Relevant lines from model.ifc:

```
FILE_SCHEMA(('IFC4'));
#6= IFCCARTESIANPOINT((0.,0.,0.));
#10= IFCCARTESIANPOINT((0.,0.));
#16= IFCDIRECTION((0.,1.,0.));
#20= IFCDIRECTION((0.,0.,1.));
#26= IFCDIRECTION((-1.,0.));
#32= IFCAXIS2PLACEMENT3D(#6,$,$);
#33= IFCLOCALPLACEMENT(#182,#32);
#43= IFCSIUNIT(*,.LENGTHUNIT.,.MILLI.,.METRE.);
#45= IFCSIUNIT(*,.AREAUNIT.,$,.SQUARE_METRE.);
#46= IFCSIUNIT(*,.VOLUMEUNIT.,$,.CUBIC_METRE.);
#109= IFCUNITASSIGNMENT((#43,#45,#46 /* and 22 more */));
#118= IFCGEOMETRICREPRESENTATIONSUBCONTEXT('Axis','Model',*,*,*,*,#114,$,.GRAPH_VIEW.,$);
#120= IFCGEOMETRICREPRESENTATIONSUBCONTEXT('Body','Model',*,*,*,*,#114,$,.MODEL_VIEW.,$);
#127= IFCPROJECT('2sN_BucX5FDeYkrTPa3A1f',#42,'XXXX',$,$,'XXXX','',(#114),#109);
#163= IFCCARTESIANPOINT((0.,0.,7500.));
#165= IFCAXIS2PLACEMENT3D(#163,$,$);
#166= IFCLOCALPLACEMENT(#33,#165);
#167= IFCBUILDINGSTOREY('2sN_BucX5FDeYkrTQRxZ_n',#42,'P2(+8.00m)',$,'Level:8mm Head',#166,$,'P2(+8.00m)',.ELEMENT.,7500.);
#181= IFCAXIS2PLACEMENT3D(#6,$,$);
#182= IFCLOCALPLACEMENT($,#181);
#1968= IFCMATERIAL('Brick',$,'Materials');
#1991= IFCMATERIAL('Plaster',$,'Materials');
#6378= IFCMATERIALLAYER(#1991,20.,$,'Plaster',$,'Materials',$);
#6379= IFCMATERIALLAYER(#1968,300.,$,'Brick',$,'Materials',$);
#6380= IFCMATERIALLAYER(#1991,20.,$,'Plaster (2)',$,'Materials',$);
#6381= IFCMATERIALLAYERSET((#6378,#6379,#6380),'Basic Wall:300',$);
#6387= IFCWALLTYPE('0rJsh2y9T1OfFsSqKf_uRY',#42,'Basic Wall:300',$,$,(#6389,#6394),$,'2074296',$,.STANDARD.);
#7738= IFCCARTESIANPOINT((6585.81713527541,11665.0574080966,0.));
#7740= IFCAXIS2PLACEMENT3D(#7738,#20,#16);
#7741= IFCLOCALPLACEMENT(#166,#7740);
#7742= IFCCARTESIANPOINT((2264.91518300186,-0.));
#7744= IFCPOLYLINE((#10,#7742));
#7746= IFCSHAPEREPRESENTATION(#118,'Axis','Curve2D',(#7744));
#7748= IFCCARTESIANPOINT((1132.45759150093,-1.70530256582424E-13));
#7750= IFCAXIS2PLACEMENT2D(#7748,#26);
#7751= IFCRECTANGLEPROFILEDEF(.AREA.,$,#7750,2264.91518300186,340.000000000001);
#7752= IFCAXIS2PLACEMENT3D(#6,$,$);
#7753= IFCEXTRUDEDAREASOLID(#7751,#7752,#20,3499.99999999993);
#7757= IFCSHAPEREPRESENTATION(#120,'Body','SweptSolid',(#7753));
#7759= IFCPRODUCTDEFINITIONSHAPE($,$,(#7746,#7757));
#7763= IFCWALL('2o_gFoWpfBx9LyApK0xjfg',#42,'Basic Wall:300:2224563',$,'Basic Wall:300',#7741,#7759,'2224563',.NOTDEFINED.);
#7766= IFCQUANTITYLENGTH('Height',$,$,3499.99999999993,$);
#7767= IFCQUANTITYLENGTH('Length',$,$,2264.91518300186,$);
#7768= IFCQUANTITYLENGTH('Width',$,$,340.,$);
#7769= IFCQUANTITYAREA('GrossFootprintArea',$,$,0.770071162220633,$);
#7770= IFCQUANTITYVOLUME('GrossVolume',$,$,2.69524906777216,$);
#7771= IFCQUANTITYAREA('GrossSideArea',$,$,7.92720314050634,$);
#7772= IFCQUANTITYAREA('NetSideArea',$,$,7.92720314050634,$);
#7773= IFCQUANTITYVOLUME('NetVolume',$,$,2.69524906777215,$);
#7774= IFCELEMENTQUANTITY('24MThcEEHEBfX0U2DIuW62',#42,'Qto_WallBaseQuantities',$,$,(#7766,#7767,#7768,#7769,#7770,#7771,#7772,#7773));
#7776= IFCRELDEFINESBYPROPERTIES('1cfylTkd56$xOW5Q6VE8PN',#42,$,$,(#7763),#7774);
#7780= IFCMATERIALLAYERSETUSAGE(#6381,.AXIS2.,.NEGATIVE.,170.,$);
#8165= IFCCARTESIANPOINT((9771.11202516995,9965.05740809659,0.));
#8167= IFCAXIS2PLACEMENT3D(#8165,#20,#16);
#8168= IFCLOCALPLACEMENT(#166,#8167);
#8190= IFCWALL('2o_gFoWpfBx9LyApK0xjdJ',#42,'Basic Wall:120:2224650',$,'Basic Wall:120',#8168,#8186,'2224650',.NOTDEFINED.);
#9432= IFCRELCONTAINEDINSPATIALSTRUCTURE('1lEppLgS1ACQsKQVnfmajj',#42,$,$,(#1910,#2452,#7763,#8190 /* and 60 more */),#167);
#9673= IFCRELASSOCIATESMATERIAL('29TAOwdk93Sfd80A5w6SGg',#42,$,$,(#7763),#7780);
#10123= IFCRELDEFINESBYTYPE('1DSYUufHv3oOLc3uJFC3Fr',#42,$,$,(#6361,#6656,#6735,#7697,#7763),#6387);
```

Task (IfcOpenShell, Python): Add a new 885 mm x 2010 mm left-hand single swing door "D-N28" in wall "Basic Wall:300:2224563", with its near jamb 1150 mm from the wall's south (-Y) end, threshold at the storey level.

```python
import numpy as np
import ifcopenshell
import ifcopenshell.api.feature
import ifcopenshell.api.geometry
import ifcopenshell.api.pset
import ifcopenshell.api.root
import ifcopenshell.api.spatial
import ifcopenshell.geom
import ifcopenshell.util.element
import ifcopenshell.util.placement
import ifcopenshell.util.representation
import ifcopenshell.util.shape
import ifcopenshell.util.unit

model = ifcopenshell.open("model.ifc")
unit_scale = ifcopenshell.util.unit.calculate_unit_scale(model)
area_scale = ifcopenshell.util.unit.calculate_unit_scale(model, "AREAUNIT")
volume_scale = ifcopenshell.util.unit.calculate_unit_scale(model, "VOLUMEUNIT")
settings = ifcopenshell.geom.settings()


def volume(element):
    """Net volume in cubic metres, openings subtracted."""
    shape = ifcopenshell.geom.create_shape(settings, element)
    return ifcopenshell.util.shape.get_volume(shape.geometry)


wall = model.by_guid("2o_gFoWpfBx9LyApK0xjfg")
storey = ifcopenshell.util.element.get_container(wall, ifc_class="IfcBuildingStorey")
context = ifcopenshell.util.representation.get_context(model, "Model", "Body", "MODEL_VIEW")
before = volume(wall)

width, height, from_end, sill = 0.885, 2.01, 1.15, 0.0  # metres

# The wall runs along its own X axis, and the end named is its -X end.
wall_shape = ifcopenshell.geom.create_shape(settings, wall)
x, y, z = ifcopenshell.util.shape.get_vertices(wall_shape.geometry).T
start = x.min() + from_end
face, thickness = float(y.min()), float(y.max() - y.min())
wall_matrix = ifcopenshell.util.placement.get_local_placement(wall.ObjectPlacement)
level = ifcopenshell.util.placement.get_local_placement(storey.ObjectPlacement)[2, 3]


def in_wall(x, y):
    """Placement at x, y metres in the wall's axes, at sill height."""
    matrix = wall_matrix.copy()
    matrix[:, 3] = wall_matrix @ np.array([x / unit_scale, y / unit_scale, 0.0, 1.0])
    matrix[2, 3] = level + sill / unit_scale
    return matrix


# Opening: a box that overshoots both wall faces by 50 mm.
opening = ifcopenshell.api.root.create_entity(model, ifc_class="IfcOpeningElement", predefined_type="OPENING")
box = ifcopenshell.api.geometry.add_wall_representation(
    model, context=context, length=width, height=height, thickness=thickness + 0.1
)
ifcopenshell.api.geometry.assign_representation(model, product=opening, representation=box)
ifcopenshell.api.geometry.edit_object_placement(model, product=opening, matrix=in_wall(start, face - 0.05), is_si=False)
ifcopenshell.api.feature.add_feature(model, feature=opening, element=wall)

door = ifcopenshell.api.root.create_entity(model, ifc_class="IfcDoor", name="D-N28", predefined_type="DOOR")
door.OverallWidth, door.OverallHeight = width / unit_scale, height / unit_scale
door.OperationType = "SINGLE_SWING_LEFT"
body = ifcopenshell.api.geometry.add_door_representation(
    model,
    context=context,
    overall_width=door.OverallWidth,
    overall_height=door.OverallHeight,
    operation_type="SINGLE_SWING_LEFT",
    lining_properties={"LiningDepth": thickness / unit_scale, "ThresholdDepth": thickness / unit_scale},
)
ifcopenshell.api.geometry.assign_representation(model, product=door, representation=body)
ifcopenshell.api.spatial.assign_container(model, products=[door], relating_structure=storey)
ifcopenshell.api.feature.add_filling(model, opening=opening, element=door)

# The lining spans the wall, so the door starts at the wall face.
ifcopenshell.api.geometry.edit_object_placement(model, product=door, matrix=in_wall(start, face), is_si=False)

after = volume(wall)

# Update the wall's stored quantities.
qto = model.by_id(ifcopenshell.util.element.get_pset(wall, "Qto_WallBaseQuantities", should_inherit=False)["id"])
ifcopenshell.api.pset.edit_qto(model, qto=qto, properties={
    "NetSideArea": after / thickness / area_scale,
    "NetVolume": after / volume_scale,
})

print(f"wall volume {before:.3f} -> {after:.3f} m3")

model.write("model_edited.ifc")
```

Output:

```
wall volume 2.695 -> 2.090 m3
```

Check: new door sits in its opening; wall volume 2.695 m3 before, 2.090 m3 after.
